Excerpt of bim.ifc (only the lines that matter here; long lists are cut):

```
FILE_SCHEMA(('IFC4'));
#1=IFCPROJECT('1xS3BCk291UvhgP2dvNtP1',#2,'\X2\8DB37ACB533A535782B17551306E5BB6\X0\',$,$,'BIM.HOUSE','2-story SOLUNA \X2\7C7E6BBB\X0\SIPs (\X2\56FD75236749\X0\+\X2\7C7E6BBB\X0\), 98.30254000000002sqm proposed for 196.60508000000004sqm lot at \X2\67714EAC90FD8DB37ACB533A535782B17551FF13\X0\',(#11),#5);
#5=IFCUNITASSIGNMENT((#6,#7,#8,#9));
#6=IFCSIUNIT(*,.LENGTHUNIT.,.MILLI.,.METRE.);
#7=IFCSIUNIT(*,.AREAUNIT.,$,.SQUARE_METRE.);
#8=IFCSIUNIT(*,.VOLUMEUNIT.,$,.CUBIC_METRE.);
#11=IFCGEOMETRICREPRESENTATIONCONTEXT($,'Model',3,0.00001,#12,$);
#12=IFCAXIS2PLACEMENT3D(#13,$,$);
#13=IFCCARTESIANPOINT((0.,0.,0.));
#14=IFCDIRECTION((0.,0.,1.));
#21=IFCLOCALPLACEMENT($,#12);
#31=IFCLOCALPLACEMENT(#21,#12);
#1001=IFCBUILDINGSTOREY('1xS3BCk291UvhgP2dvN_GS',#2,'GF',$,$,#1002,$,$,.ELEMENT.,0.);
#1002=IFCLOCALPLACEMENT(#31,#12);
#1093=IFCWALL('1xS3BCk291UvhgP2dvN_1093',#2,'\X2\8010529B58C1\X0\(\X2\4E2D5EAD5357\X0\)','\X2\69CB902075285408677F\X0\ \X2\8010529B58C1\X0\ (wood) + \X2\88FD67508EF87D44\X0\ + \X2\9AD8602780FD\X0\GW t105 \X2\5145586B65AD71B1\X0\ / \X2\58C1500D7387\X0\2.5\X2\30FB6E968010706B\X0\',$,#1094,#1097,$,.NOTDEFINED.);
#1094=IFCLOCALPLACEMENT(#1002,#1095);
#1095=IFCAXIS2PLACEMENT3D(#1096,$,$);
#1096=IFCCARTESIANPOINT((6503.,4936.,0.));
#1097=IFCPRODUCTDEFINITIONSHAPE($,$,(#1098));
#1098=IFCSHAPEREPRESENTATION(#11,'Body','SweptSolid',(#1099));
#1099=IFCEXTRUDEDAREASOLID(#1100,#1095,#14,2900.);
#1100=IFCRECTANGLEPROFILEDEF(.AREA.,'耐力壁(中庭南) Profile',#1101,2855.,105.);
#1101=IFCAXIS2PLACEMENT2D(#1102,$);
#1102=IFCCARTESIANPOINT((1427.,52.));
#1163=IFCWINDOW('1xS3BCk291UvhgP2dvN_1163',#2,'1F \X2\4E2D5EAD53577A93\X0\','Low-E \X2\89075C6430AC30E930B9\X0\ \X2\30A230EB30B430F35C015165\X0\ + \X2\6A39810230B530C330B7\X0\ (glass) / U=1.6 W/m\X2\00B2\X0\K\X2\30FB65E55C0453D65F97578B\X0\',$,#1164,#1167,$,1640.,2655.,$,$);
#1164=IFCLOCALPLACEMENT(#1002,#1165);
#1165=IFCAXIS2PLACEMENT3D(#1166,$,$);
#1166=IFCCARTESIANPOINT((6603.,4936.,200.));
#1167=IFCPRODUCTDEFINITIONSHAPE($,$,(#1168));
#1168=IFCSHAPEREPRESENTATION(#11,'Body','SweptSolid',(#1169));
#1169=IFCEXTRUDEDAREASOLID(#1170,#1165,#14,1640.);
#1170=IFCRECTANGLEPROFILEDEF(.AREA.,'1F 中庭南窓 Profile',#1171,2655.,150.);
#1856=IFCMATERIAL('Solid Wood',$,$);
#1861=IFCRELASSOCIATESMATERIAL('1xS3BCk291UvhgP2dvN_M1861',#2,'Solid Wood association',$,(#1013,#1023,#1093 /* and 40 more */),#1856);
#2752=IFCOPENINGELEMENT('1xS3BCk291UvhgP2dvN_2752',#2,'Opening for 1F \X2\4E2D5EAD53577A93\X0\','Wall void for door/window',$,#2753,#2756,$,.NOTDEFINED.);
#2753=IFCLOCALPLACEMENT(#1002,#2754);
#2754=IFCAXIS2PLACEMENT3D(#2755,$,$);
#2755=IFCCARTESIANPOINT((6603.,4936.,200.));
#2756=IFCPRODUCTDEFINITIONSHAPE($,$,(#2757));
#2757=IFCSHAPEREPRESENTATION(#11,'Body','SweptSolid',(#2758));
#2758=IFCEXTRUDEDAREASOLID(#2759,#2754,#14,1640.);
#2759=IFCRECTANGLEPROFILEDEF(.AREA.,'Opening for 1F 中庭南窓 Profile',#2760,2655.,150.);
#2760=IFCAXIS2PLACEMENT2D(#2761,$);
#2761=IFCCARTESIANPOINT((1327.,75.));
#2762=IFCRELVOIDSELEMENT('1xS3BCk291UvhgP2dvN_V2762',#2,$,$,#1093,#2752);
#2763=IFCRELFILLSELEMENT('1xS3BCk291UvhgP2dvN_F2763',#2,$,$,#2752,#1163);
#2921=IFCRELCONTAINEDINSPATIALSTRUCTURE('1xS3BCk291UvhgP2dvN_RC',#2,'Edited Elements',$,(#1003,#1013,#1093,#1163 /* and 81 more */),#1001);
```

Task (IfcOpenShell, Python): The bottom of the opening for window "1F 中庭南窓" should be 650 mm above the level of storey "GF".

```python
import numpy as np
import ifcopenshell
import ifcopenshell.api.geometry
import ifcopenshell.geom
import ifcopenshell.util.element
import ifcopenshell.util.placement
import ifcopenshell.util.shape
import ifcopenshell.util.unit

model = ifcopenshell.open("bim.ifc")
unit_scale = ifcopenshell.util.unit.calculate_unit_scale(model)

window = model.by_guid("1xS3BCk291UvhgP2dvN_1163")
opening = window.FillsVoids[0].RelatingOpeningElement
storey = ifcopenshell.util.element.get_container(window, ifc_class="IfcBuildingStorey")
level = ifcopenshell.util.placement.get_local_placement(storey.ObjectPlacement)[2, 3]

# The opening's origin need not be at the sill, so measure its lowest point.
shape = ifcopenshell.geom.create_shape(ifcopenshell.geom.settings(), opening)
bottom = ifcopenshell.util.shape.get_shape_bottom_elevation(shape, shape.geometry) / unit_scale
dz = level + 0.65 / unit_scale - bottom

shift = np.array([0.0, 0.0, dz])
# The window is not placed relative to its opening, so move both.
for product in (opening, window):
    matrix = ifcopenshell.util.placement.get_local_placement(product.ObjectPlacement)
    matrix[:3, 3] += shift
    ifcopenshell.api.geometry.edit_object_placement(model, product=product, matrix=matrix, is_si=False)

print(f"moved by {dz * unit_scale:+.3f} m")

model.write("bim_rev.ifc")
```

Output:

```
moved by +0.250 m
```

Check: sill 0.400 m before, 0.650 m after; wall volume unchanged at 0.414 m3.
